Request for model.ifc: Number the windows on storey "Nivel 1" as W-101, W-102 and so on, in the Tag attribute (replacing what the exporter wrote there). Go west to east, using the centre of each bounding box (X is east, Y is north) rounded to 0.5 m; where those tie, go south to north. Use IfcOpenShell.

First a look at what the model holds.

```python
import ifcopenshell
import ifcopenshell.util.element
import ifcopenshell.util.placement

model = ifcopenshell.open("model.ifc")
print(model.schema)
storey = next(s for s in model.by_type("IfcBuildingStorey") if s.Name == "Nivel 1")
windows = [e for e in ifcopenshell.util.element.get_decomposition(storey) if e.is_a("IfcWindow")]
for e in sorted(windows, key=lambda e: e.id()):
    origin = ifcopenshell.util.placement.get_local_placement(e.ObjectPlacement)[:3, 3]
    print(e.id(), e.Tag, e.Name, origin.round(2) + 0.0, sep=" | ")
```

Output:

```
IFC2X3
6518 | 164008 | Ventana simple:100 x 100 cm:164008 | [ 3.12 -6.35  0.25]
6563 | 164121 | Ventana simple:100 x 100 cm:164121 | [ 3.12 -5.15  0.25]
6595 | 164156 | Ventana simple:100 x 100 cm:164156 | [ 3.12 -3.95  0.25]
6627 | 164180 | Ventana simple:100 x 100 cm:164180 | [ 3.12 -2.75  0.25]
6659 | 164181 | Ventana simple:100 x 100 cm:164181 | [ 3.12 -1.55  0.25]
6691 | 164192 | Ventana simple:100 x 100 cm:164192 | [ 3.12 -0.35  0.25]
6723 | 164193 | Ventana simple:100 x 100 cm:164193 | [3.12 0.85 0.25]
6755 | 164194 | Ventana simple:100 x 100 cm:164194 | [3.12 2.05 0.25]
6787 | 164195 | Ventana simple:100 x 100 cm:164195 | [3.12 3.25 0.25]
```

```python
import ifcopenshell
import ifcopenshell.geom
import ifcopenshell.util.element
import ifcopenshell.util.shape

model = ifcopenshell.open("model.ifc")
settings = ifcopenshell.geom.settings()
settings.set("use-world-coords", True)


def centre(element):
    shape = ifcopenshell.geom.create_shape(settings, element)
    return ifcopenshell.util.shape.get_bbox_centroid(shape.geometry)


storey = next(s for s in model.by_type("IfcBuildingStorey") if s.Name == "Nivel 1")
windows = [e for e in ifcopenshell.util.element.get_decomposition(storey) if e.is_a("IfcWindow")]

# Insertion points can sit at a corner or the storey origin, so sort by the geometry (in metres).
centres = {e: centre(e) for e in windows}
windows.sort(key=lambda e: (round(centres[e][0] / 0.5), centres[e][1]))

for i, e in enumerate(windows, start=1):
    number = f"W-1{i:02d}"
    e.Tag = number
    print(e.id(), number)

model.write("model-out.ifc")
```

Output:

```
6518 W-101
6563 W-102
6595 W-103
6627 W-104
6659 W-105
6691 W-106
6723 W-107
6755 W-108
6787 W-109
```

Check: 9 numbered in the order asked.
